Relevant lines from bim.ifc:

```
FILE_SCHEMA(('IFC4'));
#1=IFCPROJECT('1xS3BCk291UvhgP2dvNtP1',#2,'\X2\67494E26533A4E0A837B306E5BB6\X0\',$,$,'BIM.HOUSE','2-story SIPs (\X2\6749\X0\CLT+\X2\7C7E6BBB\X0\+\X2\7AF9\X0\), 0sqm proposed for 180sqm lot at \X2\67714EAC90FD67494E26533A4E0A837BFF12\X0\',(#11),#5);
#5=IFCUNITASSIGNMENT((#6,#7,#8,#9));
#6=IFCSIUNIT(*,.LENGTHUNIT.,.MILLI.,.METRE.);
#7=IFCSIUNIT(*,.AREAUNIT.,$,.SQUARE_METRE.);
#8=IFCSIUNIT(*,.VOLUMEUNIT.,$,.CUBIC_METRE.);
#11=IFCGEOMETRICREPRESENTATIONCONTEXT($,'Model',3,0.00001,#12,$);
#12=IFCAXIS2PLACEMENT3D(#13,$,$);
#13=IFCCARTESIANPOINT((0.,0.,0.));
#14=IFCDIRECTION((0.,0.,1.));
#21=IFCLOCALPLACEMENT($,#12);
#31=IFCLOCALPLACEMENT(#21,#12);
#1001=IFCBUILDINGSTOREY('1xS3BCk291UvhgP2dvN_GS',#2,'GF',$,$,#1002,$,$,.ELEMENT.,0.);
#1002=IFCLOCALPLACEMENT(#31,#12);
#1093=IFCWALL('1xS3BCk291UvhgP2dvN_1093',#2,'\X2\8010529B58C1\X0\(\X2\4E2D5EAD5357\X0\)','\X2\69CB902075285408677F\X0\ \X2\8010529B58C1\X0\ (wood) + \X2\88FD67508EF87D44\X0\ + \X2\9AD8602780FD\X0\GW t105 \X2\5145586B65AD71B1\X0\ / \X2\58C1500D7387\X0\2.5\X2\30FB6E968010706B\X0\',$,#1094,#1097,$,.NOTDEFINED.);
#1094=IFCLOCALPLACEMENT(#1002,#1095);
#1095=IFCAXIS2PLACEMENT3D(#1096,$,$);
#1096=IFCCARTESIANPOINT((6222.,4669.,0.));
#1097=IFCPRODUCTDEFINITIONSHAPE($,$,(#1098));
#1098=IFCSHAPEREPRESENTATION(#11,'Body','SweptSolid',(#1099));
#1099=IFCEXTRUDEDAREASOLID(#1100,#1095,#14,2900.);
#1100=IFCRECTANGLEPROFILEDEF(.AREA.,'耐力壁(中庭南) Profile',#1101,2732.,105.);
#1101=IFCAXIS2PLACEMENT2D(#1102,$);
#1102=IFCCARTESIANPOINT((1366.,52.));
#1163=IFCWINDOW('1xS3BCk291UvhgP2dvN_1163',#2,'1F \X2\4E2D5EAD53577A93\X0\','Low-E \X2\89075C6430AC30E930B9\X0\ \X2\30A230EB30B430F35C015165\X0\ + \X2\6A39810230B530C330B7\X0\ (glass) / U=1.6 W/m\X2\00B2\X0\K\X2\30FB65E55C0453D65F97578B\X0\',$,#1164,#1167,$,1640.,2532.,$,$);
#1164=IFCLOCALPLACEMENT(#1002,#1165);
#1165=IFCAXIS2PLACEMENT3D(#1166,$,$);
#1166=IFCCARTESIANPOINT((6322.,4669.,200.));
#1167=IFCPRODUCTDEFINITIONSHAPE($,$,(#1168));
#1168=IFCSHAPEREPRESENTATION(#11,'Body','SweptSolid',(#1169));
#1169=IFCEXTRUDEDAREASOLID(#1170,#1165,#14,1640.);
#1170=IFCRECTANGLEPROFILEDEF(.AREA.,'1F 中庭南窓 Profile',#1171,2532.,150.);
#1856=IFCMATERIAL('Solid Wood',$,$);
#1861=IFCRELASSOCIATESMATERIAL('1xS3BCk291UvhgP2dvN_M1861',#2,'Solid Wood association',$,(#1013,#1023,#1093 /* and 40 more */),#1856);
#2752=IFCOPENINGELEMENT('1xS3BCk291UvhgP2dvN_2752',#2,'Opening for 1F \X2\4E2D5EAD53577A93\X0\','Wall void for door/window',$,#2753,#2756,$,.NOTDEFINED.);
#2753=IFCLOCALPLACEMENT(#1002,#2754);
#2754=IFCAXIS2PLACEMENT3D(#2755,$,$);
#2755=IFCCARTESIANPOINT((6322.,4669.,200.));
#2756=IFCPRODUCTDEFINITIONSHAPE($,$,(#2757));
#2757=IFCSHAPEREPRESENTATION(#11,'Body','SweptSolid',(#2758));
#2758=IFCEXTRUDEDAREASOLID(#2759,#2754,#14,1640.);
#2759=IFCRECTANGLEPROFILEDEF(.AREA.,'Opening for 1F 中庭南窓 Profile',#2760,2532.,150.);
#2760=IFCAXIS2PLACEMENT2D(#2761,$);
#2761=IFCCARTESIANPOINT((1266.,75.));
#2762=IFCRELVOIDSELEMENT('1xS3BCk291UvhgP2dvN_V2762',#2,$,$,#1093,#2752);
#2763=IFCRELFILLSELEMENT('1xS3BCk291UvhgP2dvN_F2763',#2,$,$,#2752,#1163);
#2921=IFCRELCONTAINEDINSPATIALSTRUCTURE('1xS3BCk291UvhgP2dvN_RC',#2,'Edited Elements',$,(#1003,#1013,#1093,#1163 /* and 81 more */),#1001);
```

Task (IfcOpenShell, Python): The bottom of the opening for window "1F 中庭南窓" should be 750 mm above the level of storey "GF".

```python
import numpy as np
import ifcopenshell
import ifcopenshell.api.geometry
import ifcopenshell.geom
import ifcopenshell.util.element
import ifcopenshell.util.placement
import ifcopenshell.util.shape
import ifcopenshell.util.unit

model = ifcopenshell.open("bim.ifc")
unit_scale = ifcopenshell.util.unit.calculate_unit_scale(model)

window = model.by_guid("1xS3BCk291UvhgP2dvN_1163")
opening = window.FillsVoids[0].RelatingOpeningElement
storey = ifcopenshell.util.element.get_container(window, ifc_class="IfcBuildingStorey")
level = ifcopenshell.util.placement.get_local_placement(storey.ObjectPlacement)[2, 3]

# The opening's origin need not be at the sill, so measure its lowest point.
shape = ifcopenshell.geom.create_shape(ifcopenshell.geom.settings(), opening)
bottom = ifcopenshell.util.shape.get_shape_bottom_elevation(shape, shape.geometry) / unit_scale
dz = level + 0.75 / unit_scale - bottom

shift = np.array([0.0, 0.0, dz])
# The window is not placed relative to its opening, so move both.
for product in (opening, window):
    matrix = ifcopenshell.util.placement.get_local_placement(product.ObjectPlacement)
    matrix[:3, 3] += shift
    ifcopenshell.api.geometry.edit_object_placement(model, product=product, matrix=matrix, is_si=False)

print(f"moved by {dz * unit_scale:+.3f} m")

model.write("bim_rev.ifc")
```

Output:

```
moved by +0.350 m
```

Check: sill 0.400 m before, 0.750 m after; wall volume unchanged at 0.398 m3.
